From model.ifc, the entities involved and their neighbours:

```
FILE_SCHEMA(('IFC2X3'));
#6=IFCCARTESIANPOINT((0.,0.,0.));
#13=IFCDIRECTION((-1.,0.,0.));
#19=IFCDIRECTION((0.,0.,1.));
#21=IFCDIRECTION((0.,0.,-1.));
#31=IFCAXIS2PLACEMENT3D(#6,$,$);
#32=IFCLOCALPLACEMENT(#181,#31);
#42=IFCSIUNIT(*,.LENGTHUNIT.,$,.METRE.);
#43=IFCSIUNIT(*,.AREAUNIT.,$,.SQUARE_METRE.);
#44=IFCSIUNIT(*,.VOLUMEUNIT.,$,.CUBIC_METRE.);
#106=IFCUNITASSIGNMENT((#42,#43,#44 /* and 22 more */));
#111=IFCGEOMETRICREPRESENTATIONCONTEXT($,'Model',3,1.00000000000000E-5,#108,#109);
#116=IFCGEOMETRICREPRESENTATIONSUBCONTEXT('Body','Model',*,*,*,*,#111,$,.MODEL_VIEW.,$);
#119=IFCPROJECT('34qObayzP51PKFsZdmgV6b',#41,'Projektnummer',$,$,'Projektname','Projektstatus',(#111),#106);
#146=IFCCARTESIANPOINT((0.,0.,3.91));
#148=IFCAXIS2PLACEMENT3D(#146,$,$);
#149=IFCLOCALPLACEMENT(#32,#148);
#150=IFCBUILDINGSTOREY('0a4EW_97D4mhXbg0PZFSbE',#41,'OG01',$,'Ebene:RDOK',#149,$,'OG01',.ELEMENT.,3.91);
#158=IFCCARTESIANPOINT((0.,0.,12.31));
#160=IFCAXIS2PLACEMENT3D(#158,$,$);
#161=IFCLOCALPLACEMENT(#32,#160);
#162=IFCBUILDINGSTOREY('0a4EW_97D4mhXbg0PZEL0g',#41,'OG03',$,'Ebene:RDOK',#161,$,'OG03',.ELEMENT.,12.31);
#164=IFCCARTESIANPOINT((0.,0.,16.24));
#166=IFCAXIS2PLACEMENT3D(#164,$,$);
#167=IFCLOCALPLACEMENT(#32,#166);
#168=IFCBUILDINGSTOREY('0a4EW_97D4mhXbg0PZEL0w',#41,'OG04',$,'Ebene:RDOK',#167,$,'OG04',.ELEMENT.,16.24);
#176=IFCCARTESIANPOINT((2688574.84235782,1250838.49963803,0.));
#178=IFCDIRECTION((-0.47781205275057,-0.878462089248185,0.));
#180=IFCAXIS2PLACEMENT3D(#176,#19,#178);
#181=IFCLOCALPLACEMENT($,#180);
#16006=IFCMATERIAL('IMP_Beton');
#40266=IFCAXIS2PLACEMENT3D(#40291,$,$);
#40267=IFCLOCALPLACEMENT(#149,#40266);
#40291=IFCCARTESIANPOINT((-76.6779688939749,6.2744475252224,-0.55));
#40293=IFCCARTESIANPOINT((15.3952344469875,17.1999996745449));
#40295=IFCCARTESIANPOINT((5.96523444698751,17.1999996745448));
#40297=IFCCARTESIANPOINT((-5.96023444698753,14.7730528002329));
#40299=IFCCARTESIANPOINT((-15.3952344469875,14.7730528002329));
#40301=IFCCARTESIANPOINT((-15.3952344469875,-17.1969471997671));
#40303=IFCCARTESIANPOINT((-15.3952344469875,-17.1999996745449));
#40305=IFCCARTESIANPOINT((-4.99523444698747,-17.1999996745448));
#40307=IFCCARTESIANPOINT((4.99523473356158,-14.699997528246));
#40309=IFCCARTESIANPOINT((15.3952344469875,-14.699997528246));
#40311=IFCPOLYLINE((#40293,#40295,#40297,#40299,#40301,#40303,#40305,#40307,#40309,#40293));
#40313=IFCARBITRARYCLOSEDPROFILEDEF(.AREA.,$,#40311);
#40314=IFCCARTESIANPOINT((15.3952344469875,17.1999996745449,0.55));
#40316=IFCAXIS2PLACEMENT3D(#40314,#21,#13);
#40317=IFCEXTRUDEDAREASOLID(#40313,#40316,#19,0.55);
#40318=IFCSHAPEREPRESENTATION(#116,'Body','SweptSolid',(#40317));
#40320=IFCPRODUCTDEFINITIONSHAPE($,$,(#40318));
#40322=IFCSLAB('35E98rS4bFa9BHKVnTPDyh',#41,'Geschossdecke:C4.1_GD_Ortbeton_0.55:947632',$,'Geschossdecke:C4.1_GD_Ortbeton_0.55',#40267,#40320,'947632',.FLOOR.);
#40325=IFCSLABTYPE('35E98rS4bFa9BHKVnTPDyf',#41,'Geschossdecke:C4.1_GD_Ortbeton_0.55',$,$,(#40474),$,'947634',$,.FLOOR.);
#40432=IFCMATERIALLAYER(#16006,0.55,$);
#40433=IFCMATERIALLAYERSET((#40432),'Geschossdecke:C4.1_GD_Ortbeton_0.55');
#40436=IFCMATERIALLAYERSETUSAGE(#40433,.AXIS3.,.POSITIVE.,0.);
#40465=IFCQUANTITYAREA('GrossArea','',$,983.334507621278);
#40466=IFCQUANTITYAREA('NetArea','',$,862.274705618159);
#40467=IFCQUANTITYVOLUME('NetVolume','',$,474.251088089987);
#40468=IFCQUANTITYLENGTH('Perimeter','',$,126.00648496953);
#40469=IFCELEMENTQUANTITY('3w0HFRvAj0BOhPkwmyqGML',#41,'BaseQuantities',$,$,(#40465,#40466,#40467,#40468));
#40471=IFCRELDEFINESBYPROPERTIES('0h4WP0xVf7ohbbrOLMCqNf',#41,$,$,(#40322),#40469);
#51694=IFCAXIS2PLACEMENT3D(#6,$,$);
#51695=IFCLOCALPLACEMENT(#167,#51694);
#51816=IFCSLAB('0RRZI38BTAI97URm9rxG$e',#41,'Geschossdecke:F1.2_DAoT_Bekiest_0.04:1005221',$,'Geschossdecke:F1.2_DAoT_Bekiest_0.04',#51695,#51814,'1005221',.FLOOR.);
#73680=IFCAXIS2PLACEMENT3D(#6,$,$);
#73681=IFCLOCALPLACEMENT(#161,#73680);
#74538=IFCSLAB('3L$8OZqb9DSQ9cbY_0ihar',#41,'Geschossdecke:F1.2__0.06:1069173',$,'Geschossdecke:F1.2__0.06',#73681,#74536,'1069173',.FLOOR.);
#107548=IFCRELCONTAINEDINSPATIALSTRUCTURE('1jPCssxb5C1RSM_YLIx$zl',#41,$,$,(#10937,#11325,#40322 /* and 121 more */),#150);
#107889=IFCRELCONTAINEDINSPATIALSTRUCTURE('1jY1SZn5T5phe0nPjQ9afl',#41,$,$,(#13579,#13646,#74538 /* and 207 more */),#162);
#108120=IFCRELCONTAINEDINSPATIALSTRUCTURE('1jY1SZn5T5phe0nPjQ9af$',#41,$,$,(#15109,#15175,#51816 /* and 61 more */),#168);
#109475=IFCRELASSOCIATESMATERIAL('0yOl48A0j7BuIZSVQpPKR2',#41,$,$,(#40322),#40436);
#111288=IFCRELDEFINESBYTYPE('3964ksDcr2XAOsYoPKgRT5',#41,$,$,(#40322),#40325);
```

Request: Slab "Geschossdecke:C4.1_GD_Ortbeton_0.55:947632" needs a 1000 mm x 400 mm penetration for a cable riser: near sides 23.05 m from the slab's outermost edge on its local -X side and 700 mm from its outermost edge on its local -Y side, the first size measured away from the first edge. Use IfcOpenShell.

```python
import numpy as np
import ifcopenshell
import ifcopenshell.api.feature
import ifcopenshell.api.geometry
import ifcopenshell.api.pset
import ifcopenshell.api.root
import ifcopenshell.geom
import ifcopenshell.util.element
import ifcopenshell.util.placement
import ifcopenshell.util.representation
import ifcopenshell.util.shape
import ifcopenshell.util.unit

model = ifcopenshell.open("model.ifc")
unit_scale = ifcopenshell.util.unit.calculate_unit_scale(model)
area_scale = ifcopenshell.util.unit.calculate_unit_scale(model, "AREAUNIT")
volume_scale = ifcopenshell.util.unit.calculate_unit_scale(model, "VOLUMEUNIT")
settings = ifcopenshell.geom.settings()


def volume(element):
    """Net volume in cubic metres, openings subtracted."""
    shape = ifcopenshell.geom.create_shape(settings, element)
    return ifcopenshell.util.shape.get_volume(shape.geometry)


slab = model.by_guid("35E98rS4bFa9BHKVnTPDyh")
before = volume(slab)

# Extent in the slab's own axes, in metres. The edges named are its -X and -Y sides.
slab_shape = ifcopenshell.geom.create_shape(settings, slab)
vertices = ifcopenshell.util.shape.get_vertices(slab_shape.geometry)
x_min, y_min, bottom = vertices.min(axis=0)
top = vertices[:, 2].max()

opening = ifcopenshell.api.root.create_entity(model, ifc_class="IfcOpeningElement", name="Cable riser opening")
context = ifcopenshell.util.representation.get_context(model, "Model", "Body", "MODEL_VIEW")
width, depth = 1, 0.4
outline = [(0.0, 0.0), (width, 0.0), (width, depth), (0.0, depth), (0.0, 0.0)]
# Overshoot both faces by 50 mm so the cut is clean.
shape = ifcopenshell.api.geometry.add_slab_representation(
    model, context=context, depth=top - bottom + 0.1, polyline=outline
)
ifcopenshell.api.geometry.assign_representation(model, product=opening, representation=shape)

matrix = ifcopenshell.util.placement.get_local_placement(slab.ObjectPlacement)
matrix[:, 3] = matrix @ np.append(np.array([x_min + 23.05, y_min + 0.7, bottom - 0.05]) / unit_scale, 1.0)
ifcopenshell.api.geometry.edit_object_placement(model, product=opening, matrix=matrix, is_si=False)
ifcopenshell.api.feature.add_feature(model, feature=opening, element=slab)

after = volume(slab)

# Update the slab's stored quantities.
qto = model.by_id(ifcopenshell.util.element.get_pset(slab, "BaseQuantities", should_inherit=False)["id"])
ifcopenshell.api.pset.edit_qto(model, qto=qto, properties={
    "NetArea": after / (top - bottom) / area_scale,
    "NetVolume": after / volume_scale,
})

print(f"slab volume {before:.3f} -> {after:.3f} m3")

model.write("model_rev.ifc")
```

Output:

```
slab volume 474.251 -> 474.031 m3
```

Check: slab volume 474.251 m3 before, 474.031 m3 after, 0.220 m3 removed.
